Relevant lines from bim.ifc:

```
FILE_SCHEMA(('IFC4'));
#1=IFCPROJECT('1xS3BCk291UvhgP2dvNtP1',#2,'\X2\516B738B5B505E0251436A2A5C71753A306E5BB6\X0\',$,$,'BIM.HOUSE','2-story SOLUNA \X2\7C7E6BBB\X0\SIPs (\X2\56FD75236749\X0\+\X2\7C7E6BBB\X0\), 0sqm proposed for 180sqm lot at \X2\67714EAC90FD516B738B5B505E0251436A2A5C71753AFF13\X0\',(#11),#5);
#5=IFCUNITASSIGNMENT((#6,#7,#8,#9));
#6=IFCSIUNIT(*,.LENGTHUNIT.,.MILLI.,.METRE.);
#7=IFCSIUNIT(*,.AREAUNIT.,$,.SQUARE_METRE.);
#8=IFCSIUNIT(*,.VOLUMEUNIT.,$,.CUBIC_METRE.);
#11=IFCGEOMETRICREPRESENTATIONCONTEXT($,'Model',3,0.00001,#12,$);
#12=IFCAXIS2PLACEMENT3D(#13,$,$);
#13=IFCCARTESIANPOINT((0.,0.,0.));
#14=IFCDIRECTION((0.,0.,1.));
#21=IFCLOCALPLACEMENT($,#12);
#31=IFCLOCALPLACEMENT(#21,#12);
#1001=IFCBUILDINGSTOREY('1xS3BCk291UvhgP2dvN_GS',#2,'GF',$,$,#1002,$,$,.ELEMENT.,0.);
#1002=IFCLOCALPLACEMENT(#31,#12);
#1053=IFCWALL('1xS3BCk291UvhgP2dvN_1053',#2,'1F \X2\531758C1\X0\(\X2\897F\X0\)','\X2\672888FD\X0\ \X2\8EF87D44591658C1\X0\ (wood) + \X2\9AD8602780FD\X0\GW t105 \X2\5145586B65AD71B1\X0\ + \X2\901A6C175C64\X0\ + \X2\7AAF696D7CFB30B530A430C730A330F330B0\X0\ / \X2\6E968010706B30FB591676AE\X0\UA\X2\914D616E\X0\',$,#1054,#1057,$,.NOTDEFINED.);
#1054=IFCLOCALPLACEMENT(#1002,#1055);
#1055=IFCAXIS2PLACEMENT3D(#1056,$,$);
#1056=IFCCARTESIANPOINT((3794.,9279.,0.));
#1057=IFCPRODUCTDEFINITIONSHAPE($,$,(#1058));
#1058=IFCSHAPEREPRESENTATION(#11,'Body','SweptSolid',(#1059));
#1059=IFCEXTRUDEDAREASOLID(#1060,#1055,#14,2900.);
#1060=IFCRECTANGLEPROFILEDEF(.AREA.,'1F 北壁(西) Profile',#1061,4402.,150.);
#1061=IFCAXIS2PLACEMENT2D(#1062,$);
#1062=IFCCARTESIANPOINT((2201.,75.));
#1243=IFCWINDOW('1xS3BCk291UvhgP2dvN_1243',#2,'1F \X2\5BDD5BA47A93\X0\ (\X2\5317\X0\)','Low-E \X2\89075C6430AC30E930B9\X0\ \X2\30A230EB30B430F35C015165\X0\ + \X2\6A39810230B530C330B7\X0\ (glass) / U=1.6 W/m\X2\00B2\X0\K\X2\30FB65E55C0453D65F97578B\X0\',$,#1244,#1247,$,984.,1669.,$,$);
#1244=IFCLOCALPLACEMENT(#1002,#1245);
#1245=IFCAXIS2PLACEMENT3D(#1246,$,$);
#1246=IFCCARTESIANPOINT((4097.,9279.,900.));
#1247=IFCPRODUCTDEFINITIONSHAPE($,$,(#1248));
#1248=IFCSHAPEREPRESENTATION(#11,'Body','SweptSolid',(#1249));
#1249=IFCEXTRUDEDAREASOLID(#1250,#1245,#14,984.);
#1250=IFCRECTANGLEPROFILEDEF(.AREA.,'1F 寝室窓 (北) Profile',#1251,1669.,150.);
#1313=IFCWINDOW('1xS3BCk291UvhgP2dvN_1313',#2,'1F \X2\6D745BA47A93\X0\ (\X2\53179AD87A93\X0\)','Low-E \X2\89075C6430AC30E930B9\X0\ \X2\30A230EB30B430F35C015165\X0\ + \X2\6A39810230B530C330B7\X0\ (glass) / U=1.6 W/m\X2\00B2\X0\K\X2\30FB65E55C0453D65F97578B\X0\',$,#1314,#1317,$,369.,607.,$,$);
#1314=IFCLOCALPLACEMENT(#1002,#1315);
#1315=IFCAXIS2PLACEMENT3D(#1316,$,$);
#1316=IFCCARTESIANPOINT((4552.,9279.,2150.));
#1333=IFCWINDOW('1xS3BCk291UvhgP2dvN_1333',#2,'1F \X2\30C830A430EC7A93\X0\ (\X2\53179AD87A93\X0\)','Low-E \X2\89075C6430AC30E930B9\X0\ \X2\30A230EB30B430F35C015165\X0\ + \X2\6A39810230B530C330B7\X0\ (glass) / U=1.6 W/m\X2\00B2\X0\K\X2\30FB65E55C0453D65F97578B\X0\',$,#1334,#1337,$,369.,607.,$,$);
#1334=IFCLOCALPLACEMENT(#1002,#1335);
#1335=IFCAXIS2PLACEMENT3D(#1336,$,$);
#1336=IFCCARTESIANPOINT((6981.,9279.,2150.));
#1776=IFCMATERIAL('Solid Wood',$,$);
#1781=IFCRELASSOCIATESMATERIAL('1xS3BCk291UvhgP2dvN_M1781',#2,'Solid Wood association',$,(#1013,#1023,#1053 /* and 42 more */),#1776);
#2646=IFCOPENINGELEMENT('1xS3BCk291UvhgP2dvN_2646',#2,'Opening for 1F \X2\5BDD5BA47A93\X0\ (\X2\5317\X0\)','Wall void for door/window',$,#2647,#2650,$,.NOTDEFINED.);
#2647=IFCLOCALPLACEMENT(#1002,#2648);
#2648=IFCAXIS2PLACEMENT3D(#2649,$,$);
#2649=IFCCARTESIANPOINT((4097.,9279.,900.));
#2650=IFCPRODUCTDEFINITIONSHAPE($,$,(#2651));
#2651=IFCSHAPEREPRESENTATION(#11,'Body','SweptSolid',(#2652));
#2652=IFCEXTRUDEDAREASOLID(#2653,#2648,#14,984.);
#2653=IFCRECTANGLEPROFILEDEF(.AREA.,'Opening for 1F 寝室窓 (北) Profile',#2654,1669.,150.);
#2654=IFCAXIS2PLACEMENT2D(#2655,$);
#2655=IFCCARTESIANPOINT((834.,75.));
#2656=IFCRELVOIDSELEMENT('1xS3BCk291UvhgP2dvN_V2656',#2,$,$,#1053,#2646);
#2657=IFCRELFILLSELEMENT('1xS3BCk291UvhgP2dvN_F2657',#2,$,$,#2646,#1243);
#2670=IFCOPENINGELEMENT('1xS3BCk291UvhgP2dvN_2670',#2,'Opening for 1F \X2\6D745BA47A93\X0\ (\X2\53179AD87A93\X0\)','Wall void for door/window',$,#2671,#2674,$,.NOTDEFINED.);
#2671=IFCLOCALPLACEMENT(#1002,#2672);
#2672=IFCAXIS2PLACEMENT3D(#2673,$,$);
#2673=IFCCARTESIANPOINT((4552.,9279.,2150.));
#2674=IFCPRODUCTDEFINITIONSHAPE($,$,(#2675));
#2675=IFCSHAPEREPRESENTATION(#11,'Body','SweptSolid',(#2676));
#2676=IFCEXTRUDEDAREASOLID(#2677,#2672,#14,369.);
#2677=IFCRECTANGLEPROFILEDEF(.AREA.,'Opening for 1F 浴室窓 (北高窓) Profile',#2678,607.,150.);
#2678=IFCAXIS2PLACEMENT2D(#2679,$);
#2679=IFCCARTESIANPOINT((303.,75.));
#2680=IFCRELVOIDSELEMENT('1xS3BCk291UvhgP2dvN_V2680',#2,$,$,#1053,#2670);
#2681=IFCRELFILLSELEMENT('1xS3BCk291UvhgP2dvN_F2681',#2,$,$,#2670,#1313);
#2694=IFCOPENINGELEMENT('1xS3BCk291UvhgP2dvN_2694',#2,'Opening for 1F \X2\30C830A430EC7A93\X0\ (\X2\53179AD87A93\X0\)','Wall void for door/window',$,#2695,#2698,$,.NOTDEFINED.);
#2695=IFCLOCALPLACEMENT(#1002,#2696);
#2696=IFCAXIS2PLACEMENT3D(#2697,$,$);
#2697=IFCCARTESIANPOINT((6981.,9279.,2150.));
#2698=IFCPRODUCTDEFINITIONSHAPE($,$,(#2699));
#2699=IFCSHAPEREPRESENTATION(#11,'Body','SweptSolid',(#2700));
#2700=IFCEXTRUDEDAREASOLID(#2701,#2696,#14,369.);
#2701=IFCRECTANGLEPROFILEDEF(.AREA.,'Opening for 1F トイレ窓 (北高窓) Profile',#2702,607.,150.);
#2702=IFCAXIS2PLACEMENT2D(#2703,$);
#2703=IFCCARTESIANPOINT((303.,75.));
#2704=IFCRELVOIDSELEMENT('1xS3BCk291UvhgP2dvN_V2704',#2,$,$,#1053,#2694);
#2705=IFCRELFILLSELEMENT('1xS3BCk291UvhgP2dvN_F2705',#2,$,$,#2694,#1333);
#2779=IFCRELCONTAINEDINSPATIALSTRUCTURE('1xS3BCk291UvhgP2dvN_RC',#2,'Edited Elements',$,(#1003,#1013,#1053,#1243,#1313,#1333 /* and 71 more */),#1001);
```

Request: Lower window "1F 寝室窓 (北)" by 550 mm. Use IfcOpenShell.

```python
import numpy as np
import ifcopenshell
import ifcopenshell.api.geometry
import ifcopenshell.util.placement
import ifcopenshell.util.unit

model = ifcopenshell.open("bim.ifc")
unit_scale = ifcopenshell.util.unit.calculate_unit_scale(model)

window = model.by_guid("1xS3BCk291UvhgP2dvN_1243")
opening = window.FillsVoids[0].RelatingOpeningElement
dz = -0.55 / unit_scale

shift = np.array([0.0, 0.0, dz])
# The window is not placed relative to its opening, so move both.
for product in (opening, window):
    matrix = ifcopenshell.util.placement.get_local_placement(product.ObjectPlacement)
    matrix[:3, 3] += shift
    ifcopenshell.api.geometry.edit_object_placement(model, product=product, matrix=matrix, is_si=False)

print(f"moved by {dz * unit_scale:+.3f} m")

model.write("bim_rev.ifc")
```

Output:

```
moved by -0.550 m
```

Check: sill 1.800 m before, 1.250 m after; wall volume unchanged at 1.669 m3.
